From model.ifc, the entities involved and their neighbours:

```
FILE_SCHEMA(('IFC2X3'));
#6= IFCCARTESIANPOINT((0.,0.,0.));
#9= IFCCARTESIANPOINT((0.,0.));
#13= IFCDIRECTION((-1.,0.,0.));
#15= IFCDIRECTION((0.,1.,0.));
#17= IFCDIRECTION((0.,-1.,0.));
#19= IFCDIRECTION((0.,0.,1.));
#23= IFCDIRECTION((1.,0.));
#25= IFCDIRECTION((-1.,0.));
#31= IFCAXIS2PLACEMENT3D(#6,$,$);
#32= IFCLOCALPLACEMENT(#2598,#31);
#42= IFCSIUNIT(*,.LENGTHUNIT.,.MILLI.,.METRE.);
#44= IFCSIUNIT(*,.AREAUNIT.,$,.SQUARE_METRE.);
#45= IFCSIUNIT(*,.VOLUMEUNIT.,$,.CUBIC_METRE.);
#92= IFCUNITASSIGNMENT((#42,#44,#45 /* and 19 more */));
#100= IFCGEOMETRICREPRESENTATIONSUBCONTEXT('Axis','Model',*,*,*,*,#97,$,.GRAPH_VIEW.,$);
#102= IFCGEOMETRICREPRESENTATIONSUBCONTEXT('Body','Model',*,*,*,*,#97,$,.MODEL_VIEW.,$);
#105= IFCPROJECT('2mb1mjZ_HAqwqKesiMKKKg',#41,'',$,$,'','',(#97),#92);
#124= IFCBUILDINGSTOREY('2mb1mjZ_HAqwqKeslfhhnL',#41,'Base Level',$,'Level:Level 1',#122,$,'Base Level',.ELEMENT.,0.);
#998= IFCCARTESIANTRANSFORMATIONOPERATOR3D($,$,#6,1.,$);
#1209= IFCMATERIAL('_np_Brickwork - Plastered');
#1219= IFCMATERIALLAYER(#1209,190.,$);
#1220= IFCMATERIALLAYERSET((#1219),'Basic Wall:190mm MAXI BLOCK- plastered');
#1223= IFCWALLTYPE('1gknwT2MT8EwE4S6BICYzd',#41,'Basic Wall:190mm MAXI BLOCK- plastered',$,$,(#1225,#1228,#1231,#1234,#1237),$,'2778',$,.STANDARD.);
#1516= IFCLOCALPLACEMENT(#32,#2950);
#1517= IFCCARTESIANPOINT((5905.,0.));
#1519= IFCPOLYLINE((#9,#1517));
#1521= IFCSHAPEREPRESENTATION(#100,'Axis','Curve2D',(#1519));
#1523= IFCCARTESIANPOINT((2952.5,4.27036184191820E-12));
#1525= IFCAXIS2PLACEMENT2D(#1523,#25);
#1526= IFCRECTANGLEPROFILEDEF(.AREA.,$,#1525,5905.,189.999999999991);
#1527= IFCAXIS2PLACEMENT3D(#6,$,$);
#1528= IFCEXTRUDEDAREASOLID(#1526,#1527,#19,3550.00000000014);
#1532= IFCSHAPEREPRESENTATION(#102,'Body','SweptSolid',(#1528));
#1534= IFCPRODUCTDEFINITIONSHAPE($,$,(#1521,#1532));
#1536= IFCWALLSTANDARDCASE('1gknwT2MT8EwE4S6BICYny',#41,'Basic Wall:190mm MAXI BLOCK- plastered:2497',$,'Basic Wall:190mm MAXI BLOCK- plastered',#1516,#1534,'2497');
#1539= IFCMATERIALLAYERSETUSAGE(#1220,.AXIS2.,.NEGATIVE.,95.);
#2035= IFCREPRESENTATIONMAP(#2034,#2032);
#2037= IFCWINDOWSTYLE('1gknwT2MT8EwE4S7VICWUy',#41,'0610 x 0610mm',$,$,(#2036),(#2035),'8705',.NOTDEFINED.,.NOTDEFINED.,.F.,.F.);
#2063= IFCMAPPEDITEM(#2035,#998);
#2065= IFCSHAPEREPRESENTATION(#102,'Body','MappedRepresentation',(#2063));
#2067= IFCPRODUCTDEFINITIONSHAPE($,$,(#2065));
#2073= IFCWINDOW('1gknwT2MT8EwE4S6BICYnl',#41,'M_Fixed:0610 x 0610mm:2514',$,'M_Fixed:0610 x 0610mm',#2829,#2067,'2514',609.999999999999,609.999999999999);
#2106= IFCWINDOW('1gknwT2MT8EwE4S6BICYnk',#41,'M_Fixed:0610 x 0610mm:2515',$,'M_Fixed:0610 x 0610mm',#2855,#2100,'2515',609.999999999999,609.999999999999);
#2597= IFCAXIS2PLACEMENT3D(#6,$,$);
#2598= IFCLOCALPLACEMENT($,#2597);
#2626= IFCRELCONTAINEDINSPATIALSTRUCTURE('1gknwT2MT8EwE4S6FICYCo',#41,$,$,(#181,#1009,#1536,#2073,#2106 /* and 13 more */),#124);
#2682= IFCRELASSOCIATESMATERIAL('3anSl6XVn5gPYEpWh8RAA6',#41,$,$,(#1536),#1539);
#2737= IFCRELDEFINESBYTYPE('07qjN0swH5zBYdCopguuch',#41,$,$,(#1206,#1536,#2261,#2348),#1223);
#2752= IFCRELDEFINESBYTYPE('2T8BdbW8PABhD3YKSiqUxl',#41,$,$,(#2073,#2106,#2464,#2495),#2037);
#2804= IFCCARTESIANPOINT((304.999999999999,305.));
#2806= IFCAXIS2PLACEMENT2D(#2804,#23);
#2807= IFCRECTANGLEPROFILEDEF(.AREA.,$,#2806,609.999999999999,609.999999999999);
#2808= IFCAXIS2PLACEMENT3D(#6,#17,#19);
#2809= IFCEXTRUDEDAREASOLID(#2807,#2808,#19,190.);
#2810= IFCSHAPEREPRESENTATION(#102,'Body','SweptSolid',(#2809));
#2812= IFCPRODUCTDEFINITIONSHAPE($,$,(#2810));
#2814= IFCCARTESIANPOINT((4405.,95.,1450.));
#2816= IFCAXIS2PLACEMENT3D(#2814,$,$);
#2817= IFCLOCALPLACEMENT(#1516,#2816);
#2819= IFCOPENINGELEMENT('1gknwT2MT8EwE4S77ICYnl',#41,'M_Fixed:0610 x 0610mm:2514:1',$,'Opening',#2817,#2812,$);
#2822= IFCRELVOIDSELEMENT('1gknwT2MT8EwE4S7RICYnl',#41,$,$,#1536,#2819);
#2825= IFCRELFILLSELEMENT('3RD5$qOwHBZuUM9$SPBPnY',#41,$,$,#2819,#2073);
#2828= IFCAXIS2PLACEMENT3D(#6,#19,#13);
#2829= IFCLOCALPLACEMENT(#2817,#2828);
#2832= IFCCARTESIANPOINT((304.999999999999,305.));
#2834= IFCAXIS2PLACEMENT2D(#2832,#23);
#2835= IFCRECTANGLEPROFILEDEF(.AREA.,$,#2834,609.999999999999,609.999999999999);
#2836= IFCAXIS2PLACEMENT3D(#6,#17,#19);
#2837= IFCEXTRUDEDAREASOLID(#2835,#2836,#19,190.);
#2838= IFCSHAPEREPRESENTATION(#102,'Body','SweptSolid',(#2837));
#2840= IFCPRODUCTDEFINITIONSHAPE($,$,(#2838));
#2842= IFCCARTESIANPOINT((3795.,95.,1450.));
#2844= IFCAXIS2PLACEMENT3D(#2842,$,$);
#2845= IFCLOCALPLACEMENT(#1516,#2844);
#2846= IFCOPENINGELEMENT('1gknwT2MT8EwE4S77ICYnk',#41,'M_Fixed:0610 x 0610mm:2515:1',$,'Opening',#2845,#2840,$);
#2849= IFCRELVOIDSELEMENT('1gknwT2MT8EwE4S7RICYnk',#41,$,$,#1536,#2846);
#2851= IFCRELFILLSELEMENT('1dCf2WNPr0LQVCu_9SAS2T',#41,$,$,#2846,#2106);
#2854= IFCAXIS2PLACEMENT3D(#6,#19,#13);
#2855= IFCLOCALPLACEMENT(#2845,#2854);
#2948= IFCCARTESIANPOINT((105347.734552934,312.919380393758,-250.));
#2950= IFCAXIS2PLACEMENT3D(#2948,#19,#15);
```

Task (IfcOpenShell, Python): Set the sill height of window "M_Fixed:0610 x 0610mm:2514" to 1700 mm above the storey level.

```python
import numpy as np
import ifcopenshell
import ifcopenshell.api.geometry
import ifcopenshell.geom
import ifcopenshell.util.element
import ifcopenshell.util.placement
import ifcopenshell.util.shape
import ifcopenshell.util.unit

model = ifcopenshell.open("model.ifc")
unit_scale = ifcopenshell.util.unit.calculate_unit_scale(model)

window = model.by_guid("1gknwT2MT8EwE4S6BICYnl")
opening = window.FillsVoids[0].RelatingOpeningElement
storey = ifcopenshell.util.element.get_container(window, ifc_class="IfcBuildingStorey")
level = ifcopenshell.util.placement.get_local_placement(storey.ObjectPlacement)[2, 3]

# The opening's origin need not be at the sill, so measure its lowest point.
shape = ifcopenshell.geom.create_shape(ifcopenshell.geom.settings(), opening)
bottom = ifcopenshell.util.shape.get_shape_bottom_elevation(shape, shape.geometry) / unit_scale
dz = level + 1700.0 - bottom

shift = np.array([0.0, 0.0, dz])
# The window is placed relative to its opening, so it follows when the opening moves.
matrix = ifcopenshell.util.placement.get_local_placement(opening.ObjectPlacement)
matrix[:3, 3] += shift
ifcopenshell.api.geometry.edit_object_placement(
    model, product=opening, matrix=matrix, is_si=False, should_transform_children=True
)

print(f"moved by {dz * unit_scale:+.3f} m")

model.write("model_edited.ifc")
```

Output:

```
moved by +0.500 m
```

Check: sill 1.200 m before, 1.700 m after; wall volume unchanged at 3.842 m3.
